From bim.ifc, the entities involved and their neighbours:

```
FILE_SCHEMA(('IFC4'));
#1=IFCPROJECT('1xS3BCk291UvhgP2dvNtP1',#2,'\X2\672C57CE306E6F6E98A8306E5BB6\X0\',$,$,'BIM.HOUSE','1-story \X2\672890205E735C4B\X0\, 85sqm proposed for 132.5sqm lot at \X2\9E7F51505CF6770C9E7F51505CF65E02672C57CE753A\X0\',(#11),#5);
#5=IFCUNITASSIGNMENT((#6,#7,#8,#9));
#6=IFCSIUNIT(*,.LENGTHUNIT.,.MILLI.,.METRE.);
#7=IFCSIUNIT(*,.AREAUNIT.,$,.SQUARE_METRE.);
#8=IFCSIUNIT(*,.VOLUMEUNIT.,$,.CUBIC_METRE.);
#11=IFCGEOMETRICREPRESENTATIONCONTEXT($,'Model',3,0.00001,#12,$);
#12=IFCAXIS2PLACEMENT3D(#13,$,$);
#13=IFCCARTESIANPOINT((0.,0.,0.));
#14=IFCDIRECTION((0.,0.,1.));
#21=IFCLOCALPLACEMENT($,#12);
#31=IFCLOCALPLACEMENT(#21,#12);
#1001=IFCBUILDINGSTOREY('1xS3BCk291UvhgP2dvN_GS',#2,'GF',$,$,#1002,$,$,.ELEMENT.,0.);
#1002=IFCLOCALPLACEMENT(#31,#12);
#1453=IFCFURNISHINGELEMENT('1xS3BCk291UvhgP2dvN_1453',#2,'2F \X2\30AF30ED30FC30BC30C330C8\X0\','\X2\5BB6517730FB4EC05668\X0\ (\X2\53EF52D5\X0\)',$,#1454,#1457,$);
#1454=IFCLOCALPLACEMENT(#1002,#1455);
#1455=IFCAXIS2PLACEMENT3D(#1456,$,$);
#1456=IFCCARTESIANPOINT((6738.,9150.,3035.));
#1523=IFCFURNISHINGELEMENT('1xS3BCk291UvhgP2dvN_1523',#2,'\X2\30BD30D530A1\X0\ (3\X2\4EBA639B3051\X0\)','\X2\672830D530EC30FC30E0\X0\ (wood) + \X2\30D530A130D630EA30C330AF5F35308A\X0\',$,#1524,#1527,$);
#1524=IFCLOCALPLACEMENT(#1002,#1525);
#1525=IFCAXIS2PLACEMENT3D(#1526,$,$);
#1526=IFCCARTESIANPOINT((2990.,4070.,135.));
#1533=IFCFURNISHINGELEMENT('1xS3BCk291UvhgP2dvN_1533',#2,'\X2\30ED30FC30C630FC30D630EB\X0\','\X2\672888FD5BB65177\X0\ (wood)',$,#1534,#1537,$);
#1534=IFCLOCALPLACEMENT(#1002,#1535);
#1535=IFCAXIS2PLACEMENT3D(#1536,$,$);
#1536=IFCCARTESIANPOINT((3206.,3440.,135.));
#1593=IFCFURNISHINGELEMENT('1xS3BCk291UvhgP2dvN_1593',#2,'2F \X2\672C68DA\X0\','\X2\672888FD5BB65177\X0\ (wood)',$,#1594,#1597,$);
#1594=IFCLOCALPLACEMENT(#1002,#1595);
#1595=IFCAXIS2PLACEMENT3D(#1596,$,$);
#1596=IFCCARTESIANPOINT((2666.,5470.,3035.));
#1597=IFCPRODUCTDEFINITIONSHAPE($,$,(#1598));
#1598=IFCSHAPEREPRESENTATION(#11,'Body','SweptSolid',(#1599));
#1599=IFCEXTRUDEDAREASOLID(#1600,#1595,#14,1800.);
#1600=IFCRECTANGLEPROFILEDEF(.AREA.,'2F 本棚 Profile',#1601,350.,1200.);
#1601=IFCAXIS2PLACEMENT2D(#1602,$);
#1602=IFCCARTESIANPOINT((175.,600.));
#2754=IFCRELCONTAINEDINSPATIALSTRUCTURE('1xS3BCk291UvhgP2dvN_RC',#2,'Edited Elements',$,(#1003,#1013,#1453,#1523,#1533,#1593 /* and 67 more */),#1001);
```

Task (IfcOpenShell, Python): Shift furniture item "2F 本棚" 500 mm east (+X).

```python
import ifcopenshell
import ifcopenshell.api.geometry
import ifcopenshell.util.placement

model = ifcopenshell.open("bim.ifc")

item = model.by_guid("1xS3BCk291UvhgP2dvN_1593")
matrix = ifcopenshell.util.placement.get_local_placement(item.ObjectPlacement)
matrix[0, 3] += 500.0
ifcopenshell.api.geometry.edit_object_placement(model, product=item, matrix=matrix, is_si=False)

print(ifcopenshell.util.placement.get_local_placement(item.ObjectPlacement).round(3) + 0.0)

model.write("bim_edited.ifc")
```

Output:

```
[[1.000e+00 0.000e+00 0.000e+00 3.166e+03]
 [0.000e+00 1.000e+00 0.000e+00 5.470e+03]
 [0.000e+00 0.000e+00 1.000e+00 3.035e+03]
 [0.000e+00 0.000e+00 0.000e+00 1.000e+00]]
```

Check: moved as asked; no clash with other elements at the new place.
